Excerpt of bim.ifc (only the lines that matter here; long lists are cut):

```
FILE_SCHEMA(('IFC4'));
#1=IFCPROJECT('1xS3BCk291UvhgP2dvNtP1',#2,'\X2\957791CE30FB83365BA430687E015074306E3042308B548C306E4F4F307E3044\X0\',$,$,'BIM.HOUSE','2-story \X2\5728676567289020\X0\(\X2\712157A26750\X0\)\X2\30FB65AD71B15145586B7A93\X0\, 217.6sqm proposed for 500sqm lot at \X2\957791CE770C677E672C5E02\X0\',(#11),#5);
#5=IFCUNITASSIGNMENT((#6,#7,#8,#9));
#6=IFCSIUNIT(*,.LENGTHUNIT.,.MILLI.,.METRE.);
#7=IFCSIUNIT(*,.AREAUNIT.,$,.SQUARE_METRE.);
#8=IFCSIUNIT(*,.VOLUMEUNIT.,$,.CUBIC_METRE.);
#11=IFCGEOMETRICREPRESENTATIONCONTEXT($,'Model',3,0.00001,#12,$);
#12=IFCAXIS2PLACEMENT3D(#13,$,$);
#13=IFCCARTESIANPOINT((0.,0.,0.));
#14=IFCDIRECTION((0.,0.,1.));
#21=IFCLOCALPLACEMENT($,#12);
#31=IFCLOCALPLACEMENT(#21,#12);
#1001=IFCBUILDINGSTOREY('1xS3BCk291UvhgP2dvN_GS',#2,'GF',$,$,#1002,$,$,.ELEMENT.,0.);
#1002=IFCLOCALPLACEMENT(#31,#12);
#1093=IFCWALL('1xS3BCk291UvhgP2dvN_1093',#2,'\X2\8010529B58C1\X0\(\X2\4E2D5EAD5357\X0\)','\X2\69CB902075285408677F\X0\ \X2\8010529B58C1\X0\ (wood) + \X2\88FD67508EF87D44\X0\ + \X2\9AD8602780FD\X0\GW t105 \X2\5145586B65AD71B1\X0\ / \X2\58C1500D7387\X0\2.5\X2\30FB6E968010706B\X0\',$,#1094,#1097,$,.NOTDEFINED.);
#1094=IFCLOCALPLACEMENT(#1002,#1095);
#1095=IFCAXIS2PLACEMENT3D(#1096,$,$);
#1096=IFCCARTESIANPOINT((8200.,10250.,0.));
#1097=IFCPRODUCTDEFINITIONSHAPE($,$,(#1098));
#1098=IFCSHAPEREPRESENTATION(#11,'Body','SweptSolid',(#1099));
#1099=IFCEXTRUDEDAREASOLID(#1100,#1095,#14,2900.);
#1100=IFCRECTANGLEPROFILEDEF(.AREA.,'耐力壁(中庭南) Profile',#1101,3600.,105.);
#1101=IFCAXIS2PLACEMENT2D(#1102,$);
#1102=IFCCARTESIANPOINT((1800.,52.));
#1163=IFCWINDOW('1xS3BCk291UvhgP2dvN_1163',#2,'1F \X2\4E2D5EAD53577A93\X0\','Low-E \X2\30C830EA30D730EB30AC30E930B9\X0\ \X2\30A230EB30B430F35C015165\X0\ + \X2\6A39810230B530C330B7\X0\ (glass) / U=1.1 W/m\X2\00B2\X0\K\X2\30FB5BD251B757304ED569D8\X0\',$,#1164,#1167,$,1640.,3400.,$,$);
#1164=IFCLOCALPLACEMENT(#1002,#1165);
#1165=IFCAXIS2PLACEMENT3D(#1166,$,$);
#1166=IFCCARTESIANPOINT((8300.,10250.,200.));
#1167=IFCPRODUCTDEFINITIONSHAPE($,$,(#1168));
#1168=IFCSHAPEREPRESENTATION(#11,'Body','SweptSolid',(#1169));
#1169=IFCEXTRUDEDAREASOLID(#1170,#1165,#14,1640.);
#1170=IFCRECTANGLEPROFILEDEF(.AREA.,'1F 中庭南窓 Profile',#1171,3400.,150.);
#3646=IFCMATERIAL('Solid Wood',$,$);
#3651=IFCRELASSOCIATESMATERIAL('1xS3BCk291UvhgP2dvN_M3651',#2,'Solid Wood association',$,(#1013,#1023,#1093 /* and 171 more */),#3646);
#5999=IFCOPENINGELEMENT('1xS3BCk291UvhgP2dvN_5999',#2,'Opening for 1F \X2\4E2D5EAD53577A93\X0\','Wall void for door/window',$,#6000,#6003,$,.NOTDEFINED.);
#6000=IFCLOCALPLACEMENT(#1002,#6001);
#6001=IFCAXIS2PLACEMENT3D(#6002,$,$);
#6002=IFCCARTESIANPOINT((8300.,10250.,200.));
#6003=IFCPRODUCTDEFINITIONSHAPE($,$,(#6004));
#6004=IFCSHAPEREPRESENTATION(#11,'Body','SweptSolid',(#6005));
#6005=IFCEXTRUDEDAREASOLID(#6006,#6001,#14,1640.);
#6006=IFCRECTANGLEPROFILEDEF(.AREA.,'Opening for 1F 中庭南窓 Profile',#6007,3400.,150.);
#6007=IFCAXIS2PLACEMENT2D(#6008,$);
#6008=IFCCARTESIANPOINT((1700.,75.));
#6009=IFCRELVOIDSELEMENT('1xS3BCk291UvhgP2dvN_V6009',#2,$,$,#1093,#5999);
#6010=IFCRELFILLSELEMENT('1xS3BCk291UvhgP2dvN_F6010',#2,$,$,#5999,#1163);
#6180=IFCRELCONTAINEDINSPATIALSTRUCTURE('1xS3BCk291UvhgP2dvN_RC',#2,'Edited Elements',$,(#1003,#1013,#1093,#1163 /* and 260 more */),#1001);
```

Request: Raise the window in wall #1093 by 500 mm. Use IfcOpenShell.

```python
import numpy as np
import ifcopenshell
import ifcopenshell.api.geometry
import ifcopenshell.util.placement
import ifcopenshell.util.unit

model = ifcopenshell.open("bim.ifc")
unit_scale = ifcopenshell.util.unit.calculate_unit_scale(model)

window = model.by_id(1163)
opening = window.FillsVoids[0].RelatingOpeningElement
dz = 0.5 / unit_scale

shift = np.array([0.0, 0.0, dz])
# The window is not placed relative to its opening, so move both.
for product in (opening, window):
    matrix = ifcopenshell.util.placement.get_local_placement(product.ObjectPlacement)
    matrix[:3, 3] += shift
    ifcopenshell.api.geometry.edit_object_placement(model, product=product, matrix=matrix, is_si=False)

print(f"moved by {dz * unit_scale:+.3f} m")

model.write("bim-out.ifc")
```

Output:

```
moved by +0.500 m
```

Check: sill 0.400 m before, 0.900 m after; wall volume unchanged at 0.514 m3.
